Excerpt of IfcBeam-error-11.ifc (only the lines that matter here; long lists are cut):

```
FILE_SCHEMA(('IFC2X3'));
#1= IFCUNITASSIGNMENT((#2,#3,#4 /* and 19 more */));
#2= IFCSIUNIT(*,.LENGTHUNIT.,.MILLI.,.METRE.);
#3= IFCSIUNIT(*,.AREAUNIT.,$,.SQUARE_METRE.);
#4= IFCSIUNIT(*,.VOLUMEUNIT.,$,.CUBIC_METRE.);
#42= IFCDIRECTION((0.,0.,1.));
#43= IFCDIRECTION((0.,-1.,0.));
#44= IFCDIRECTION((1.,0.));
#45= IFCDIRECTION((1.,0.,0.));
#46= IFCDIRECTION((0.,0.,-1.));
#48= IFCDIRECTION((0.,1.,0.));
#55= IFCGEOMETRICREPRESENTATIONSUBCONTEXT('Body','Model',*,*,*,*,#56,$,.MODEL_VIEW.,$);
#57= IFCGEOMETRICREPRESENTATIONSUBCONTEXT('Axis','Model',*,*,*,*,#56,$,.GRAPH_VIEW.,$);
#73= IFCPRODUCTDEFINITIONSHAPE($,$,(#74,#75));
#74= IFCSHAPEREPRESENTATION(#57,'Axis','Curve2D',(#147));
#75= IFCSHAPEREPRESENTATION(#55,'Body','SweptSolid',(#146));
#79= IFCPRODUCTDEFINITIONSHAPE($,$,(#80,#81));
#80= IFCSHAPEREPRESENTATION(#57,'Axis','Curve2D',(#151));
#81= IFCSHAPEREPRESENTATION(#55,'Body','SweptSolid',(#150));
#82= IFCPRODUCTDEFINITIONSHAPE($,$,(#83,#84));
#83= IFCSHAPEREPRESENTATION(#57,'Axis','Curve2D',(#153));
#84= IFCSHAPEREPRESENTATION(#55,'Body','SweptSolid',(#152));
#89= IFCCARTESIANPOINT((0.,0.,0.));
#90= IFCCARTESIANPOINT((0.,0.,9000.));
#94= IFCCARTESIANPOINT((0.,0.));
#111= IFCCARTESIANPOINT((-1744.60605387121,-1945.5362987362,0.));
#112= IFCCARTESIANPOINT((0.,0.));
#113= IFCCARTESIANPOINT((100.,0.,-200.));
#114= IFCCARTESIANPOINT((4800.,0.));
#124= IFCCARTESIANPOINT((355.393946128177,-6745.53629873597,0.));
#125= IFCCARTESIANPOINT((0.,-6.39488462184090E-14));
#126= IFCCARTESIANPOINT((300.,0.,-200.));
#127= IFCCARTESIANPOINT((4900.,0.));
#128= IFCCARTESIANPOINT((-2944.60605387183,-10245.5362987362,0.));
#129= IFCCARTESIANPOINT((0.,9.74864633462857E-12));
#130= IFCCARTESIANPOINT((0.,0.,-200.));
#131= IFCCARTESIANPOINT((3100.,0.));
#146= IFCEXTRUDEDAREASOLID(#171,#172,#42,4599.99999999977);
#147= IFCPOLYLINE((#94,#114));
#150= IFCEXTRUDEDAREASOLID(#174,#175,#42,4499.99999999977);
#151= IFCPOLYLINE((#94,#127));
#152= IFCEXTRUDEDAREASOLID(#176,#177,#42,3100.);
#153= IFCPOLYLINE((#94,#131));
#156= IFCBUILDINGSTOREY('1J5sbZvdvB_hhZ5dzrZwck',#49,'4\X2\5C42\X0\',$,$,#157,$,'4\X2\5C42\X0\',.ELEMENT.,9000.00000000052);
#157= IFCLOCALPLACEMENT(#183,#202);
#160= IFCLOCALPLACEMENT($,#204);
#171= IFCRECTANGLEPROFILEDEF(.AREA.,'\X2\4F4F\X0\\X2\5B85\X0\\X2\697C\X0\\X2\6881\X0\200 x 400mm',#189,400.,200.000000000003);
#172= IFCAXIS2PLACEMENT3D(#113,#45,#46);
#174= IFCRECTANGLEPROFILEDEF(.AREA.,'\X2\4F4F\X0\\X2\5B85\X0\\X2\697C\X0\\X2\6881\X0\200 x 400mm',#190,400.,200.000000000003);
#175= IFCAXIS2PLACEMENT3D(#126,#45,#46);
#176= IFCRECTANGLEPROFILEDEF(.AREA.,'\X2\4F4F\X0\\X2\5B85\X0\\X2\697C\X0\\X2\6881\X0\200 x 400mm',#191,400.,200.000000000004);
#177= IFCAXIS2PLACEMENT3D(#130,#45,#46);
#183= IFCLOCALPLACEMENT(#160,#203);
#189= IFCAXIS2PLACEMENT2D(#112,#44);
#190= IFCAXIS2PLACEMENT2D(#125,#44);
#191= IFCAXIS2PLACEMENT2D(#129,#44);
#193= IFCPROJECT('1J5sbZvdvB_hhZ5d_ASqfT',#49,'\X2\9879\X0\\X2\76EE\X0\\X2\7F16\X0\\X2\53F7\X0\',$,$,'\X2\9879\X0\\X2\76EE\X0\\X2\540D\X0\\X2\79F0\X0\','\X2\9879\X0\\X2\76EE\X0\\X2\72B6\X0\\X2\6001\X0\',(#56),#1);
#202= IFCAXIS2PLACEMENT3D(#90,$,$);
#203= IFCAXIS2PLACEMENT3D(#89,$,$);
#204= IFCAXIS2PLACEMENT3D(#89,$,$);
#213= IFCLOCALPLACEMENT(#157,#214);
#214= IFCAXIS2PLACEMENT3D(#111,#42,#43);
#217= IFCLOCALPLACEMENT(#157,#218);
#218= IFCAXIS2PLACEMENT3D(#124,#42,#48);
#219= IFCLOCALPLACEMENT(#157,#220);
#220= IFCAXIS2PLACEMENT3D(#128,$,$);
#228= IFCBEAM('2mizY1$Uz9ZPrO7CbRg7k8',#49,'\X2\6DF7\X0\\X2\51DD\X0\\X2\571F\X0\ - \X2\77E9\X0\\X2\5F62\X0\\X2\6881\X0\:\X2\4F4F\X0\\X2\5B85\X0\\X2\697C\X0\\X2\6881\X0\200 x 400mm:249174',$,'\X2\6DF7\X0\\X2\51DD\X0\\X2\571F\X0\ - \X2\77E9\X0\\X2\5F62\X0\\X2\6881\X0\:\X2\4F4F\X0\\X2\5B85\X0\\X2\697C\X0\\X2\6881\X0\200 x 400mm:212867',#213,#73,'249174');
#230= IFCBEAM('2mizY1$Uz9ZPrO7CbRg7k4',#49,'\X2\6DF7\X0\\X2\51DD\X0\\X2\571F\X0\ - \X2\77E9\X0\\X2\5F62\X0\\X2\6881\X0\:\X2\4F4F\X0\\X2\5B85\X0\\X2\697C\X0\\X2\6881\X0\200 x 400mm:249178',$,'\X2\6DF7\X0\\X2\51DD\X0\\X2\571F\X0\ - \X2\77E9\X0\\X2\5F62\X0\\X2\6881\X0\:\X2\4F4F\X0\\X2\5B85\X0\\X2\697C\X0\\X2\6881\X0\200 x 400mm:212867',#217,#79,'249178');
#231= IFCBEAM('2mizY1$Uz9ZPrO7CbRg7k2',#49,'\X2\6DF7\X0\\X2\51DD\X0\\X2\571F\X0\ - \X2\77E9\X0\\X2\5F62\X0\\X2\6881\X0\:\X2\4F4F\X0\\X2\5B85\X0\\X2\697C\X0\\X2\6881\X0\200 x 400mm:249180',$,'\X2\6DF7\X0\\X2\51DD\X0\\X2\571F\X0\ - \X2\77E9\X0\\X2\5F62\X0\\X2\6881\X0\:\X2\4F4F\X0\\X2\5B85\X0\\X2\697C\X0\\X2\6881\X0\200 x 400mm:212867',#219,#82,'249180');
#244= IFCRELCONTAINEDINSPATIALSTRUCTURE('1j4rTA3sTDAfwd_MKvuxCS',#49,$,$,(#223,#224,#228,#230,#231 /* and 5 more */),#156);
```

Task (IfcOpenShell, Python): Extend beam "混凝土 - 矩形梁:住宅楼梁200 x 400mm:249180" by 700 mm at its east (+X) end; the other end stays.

```python
import numpy as np
import ifcopenshell
import ifcopenshell.util.representation
import ifcopenshell.util.unit

model = ifcopenshell.open("IfcBeam-error-11.ifc")
unit_scale = ifcopenshell.util.unit.calculate_unit_scale(model)

member = model.by_guid("2mizY1$Uz9ZPrO7CbRg7k2")
change = 0.7 / unit_scale

# The extrusion runs towards the end named, so only its depth changes.
body = ifcopenshell.util.representation.get_representation(member, "Model", "Body")
solid = body.Items[0]
old_length = solid.Depth
solid.Depth += change

# Move the axis end point with it.
axis = next(r for r in member.Representation.Representations if r.RepresentationIdentifier == "Axis").Items[0]
start, end = (np.array(p.Coordinates) for p in axis.Points)
end = end + (end - start) / np.linalg.norm(end - start) * change
point = model.createIfcCartesianPoint(end.tolist())
axis.Points = [axis.Points[0], point]

print(f"length {old_length:g} -> {solid.Depth:g}")

model.write("IfcBeam-error-11_rev.ifc")
```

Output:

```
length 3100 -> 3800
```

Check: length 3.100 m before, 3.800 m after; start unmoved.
